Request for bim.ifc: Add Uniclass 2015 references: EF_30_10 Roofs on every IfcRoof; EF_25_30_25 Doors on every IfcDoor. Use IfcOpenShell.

First a look at what the model holds.

```python
import ifcopenshell

model = ifcopenshell.open("bim.ifc")
print(model.schema)
print("classifications:", [c.Name for c in model.by_type("IfcClassification")])
for ifc_class in ("IfcDoor", "IfcRoof", "IfcStair", "IfcWall", "IfcWindow"):
    print(ifc_class, len(model.by_type(ifc_class)))
```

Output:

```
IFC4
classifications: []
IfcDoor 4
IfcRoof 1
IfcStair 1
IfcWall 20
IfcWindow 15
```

```python
import ifcopenshell
import ifcopenshell.api.classification

model = ifcopenshell.open("bim.ifc")

system = ifcopenshell.api.classification.add_classification(model, classification="Uniclass 2015")

codes = {
    "IfcRoof": ("EF_30_10", "Roofs"),
    "IfcDoor": ("EF_25_30_25", "Doors"),
}
for ifc_class, (code, name) in codes.items():
    products = model.by_type(ifc_class)
    ifcopenshell.api.classification.add_reference(
        model, products=products, classification=system, identification=code, name=name
    )
    print(code, len(products))

model.write("bim_rev.ifc")
```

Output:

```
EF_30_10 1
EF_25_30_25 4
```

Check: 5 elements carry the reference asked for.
